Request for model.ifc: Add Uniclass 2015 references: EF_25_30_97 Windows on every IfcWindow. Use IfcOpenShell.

First a look at what the model holds.

```python
import ifcopenshell

model = ifcopenshell.open("model.ifc")
print(model.schema)
print("classifications:", [c.Name for c in model.by_type("IfcClassification")])
for ifc_class in ("IfcDoor", "IfcRoof", "IfcStair", "IfcWall", "IfcWindow"):
    print(ifc_class, len(model.by_type(ifc_class)))
```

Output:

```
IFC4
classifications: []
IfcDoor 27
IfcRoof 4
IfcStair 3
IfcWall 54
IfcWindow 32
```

```python
import ifcopenshell
import ifcopenshell.api.classification

model = ifcopenshell.open("model.ifc")

system = ifcopenshell.api.classification.add_classification(model, classification="Uniclass 2015")

codes = {
    "IfcWindow": ("EF_25_30_97", "Windows"),
}
for ifc_class, (code, name) in codes.items():
    products = model.by_type(ifc_class)
    ifcopenshell.api.classification.add_reference(
        model, products=products, classification=system, identification=code, name=name
    )
    print(code, len(products))

model.write("model_updated.ifc")
```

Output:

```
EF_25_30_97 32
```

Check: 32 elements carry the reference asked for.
